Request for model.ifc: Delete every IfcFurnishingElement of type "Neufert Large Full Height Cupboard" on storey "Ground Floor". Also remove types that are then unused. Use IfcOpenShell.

First a look at what the model holds.

```python
import ifcopenshell
import ifcopenshell.util.element

model = ifcopenshell.open("model.ifc")
print(model.schema)
storey = next(s for s in model.by_type("IfcBuildingStorey") if s.Name == "Ground Floor")
furniture = [e for e in ifcopenshell.util.element.get_decomposition(storey) if e.is_a("IfcFurnishingElement")]
seen = {}
for e in furniture:
    element_type = ifcopenshell.util.element.get_type(e)
    name = element_type.Name if element_type not in (None, e) else None
    seen[name] = seen.get(name, 0) + 1
for name, count in sorted(seen.items(), key=str):
    print(count, "x", name)
```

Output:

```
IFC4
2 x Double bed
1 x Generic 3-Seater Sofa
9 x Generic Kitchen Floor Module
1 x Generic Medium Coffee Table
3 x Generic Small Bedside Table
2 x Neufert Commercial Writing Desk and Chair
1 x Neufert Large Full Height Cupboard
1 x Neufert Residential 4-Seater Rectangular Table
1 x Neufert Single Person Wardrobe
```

```python
import ifcopenshell
import ifcopenshell.api.root
import ifcopenshell.util.element

model = ifcopenshell.open("model.ifc")

storey = next(s for s in model.by_type("IfcBuildingStorey") if s.Name == "Ground Floor")
furniture = [e for e in ifcopenshell.util.element.get_decomposition(storey) if e.is_a("IfcFurnishingElement")]
targets = [e for e in furniture if (t := ifcopenshell.util.element.get_type(e)) not in (None, e) and t.Name == "Neufert Large Full Height Cupboard"]
types = {ifcopenshell.util.element.get_type(e) for e in targets} - {None, *targets}

for e in targets:
    ifcopenshell.api.root.remove_product(model, product=e)
print(len(targets), "removed")

unused = [t for t in types if not ifcopenshell.util.element.get_types(t)]
for t in unused:
    ifcopenshell.api.root.remove_product(model, product=t)
print(len(unused), "unused types removed")

model.write("model_updated.ifc")
```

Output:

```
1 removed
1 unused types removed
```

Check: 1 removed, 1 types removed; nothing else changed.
